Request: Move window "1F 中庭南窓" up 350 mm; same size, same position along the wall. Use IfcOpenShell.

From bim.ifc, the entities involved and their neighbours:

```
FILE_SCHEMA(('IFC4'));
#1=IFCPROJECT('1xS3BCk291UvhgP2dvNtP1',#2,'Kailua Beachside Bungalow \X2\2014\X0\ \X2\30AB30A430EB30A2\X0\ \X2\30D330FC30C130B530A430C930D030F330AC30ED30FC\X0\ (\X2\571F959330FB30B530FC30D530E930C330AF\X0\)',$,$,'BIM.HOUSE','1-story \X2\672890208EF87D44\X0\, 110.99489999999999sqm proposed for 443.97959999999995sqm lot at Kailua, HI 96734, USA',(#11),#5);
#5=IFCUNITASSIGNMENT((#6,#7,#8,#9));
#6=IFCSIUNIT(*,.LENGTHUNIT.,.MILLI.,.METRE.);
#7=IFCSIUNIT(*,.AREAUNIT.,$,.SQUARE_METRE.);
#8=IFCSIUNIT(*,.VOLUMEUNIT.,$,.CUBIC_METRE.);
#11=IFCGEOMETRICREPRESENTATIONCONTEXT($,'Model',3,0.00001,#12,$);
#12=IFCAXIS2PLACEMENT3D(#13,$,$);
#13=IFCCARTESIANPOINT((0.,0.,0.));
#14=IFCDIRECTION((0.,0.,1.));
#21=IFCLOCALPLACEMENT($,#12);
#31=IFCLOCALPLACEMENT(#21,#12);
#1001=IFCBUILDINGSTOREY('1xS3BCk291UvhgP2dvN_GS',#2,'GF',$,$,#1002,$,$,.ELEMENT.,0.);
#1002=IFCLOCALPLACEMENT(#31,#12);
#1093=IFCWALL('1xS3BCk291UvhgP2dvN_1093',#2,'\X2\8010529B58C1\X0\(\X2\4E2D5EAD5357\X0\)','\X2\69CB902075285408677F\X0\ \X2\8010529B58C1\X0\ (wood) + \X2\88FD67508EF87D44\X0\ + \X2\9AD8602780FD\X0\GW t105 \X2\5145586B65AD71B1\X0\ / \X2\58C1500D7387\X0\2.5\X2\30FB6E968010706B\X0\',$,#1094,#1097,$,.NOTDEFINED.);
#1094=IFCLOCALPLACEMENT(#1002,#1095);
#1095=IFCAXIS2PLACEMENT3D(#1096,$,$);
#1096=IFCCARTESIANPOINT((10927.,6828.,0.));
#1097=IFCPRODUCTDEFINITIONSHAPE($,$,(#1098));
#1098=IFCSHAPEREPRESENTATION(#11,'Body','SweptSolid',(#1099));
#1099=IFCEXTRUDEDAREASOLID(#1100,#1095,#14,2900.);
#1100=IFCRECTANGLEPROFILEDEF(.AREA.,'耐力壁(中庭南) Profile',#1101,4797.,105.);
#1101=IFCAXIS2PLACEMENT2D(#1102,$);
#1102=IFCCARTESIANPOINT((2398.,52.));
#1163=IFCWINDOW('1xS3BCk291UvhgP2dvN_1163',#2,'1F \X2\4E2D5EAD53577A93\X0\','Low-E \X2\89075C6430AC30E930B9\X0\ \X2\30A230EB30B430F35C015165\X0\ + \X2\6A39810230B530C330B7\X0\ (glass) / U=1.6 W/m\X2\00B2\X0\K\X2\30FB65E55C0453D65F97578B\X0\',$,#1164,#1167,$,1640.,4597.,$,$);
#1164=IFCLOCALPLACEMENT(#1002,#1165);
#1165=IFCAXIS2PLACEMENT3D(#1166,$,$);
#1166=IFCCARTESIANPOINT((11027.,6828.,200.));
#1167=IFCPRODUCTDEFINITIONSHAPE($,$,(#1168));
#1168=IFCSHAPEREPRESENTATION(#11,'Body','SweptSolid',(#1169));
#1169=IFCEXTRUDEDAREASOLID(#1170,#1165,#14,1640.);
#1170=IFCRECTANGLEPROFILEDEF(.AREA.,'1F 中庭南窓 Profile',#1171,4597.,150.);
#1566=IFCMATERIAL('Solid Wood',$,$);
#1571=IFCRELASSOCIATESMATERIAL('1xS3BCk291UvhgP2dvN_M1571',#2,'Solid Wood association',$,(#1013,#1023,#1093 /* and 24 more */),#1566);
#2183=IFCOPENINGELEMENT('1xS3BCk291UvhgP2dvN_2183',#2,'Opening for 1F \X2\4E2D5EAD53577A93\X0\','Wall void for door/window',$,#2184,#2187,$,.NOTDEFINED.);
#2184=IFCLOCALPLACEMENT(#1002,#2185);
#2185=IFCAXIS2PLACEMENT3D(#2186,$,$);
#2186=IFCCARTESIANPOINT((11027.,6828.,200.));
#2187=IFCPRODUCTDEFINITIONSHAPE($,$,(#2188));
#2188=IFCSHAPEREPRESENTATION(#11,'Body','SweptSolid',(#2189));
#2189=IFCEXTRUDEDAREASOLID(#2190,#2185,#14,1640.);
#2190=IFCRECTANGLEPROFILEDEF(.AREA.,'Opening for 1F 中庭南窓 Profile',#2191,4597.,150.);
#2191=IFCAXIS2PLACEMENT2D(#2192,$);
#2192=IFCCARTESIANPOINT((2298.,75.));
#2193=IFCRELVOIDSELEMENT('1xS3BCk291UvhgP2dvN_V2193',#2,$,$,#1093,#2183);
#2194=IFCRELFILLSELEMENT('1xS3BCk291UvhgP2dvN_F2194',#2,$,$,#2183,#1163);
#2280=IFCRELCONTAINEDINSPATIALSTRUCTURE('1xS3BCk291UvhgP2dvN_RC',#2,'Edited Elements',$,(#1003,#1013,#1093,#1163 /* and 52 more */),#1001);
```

```python
import numpy as np
import ifcopenshell
import ifcopenshell.api.geometry
import ifcopenshell.util.placement
import ifcopenshell.util.unit

model = ifcopenshell.open("bim.ifc")
unit_scale = ifcopenshell.util.unit.calculate_unit_scale(model)

window = model.by_guid("1xS3BCk291UvhgP2dvN_1163")
opening = window.FillsVoids[0].RelatingOpeningElement
dz = 0.35 / unit_scale

shift = np.array([0.0, 0.0, dz])
# The window is not placed relative to its opening, so move both.
for product in (opening, window):
    matrix = ifcopenshell.util.placement.get_local_placement(product.ObjectPlacement)
    matrix[:3, 3] += shift
    ifcopenshell.api.geometry.edit_object_placement(model, product=product, matrix=matrix, is_si=False)

print(f"moved by {dz * unit_scale:+.3f} m")

model.write("bim_v2.ifc")
```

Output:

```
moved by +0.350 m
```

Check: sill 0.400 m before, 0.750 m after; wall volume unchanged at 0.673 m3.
